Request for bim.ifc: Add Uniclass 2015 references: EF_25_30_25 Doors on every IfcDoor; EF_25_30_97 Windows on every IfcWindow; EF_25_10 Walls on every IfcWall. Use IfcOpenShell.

First a look at what the model holds.

```python
import ifcopenshell

model = ifcopenshell.open("bim.ifc")
print(model.schema)
print("classifications:", [c.Name for c in model.by_type("IfcClassification")])
for ifc_class in ("IfcDoor", "IfcRoof", "IfcStair", "IfcWall", "IfcWindow"):
    print(ifc_class, len(model.by_type(ifc_class)))
```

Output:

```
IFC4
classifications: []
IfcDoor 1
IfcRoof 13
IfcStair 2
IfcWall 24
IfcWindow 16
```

```python
import ifcopenshell
import ifcopenshell.api.classification

model = ifcopenshell.open("bim.ifc")

system = ifcopenshell.api.classification.add_classification(model, classification="Uniclass 2015")

codes = {
    "IfcDoor": ("EF_25_30_25", "Doors"),
    "IfcWindow": ("EF_25_30_97", "Windows"),
    "IfcWall": ("EF_25_10", "Walls"),
}
for ifc_class, (code, name) in codes.items():
    products = model.by_type(ifc_class)
    ifcopenshell.api.classification.add_reference(
        model, products=products, classification=system, identification=code, name=name
    )
    print(code, len(products))

model.write("bim_rev.ifc")
```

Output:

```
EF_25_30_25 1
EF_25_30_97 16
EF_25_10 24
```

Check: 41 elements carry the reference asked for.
